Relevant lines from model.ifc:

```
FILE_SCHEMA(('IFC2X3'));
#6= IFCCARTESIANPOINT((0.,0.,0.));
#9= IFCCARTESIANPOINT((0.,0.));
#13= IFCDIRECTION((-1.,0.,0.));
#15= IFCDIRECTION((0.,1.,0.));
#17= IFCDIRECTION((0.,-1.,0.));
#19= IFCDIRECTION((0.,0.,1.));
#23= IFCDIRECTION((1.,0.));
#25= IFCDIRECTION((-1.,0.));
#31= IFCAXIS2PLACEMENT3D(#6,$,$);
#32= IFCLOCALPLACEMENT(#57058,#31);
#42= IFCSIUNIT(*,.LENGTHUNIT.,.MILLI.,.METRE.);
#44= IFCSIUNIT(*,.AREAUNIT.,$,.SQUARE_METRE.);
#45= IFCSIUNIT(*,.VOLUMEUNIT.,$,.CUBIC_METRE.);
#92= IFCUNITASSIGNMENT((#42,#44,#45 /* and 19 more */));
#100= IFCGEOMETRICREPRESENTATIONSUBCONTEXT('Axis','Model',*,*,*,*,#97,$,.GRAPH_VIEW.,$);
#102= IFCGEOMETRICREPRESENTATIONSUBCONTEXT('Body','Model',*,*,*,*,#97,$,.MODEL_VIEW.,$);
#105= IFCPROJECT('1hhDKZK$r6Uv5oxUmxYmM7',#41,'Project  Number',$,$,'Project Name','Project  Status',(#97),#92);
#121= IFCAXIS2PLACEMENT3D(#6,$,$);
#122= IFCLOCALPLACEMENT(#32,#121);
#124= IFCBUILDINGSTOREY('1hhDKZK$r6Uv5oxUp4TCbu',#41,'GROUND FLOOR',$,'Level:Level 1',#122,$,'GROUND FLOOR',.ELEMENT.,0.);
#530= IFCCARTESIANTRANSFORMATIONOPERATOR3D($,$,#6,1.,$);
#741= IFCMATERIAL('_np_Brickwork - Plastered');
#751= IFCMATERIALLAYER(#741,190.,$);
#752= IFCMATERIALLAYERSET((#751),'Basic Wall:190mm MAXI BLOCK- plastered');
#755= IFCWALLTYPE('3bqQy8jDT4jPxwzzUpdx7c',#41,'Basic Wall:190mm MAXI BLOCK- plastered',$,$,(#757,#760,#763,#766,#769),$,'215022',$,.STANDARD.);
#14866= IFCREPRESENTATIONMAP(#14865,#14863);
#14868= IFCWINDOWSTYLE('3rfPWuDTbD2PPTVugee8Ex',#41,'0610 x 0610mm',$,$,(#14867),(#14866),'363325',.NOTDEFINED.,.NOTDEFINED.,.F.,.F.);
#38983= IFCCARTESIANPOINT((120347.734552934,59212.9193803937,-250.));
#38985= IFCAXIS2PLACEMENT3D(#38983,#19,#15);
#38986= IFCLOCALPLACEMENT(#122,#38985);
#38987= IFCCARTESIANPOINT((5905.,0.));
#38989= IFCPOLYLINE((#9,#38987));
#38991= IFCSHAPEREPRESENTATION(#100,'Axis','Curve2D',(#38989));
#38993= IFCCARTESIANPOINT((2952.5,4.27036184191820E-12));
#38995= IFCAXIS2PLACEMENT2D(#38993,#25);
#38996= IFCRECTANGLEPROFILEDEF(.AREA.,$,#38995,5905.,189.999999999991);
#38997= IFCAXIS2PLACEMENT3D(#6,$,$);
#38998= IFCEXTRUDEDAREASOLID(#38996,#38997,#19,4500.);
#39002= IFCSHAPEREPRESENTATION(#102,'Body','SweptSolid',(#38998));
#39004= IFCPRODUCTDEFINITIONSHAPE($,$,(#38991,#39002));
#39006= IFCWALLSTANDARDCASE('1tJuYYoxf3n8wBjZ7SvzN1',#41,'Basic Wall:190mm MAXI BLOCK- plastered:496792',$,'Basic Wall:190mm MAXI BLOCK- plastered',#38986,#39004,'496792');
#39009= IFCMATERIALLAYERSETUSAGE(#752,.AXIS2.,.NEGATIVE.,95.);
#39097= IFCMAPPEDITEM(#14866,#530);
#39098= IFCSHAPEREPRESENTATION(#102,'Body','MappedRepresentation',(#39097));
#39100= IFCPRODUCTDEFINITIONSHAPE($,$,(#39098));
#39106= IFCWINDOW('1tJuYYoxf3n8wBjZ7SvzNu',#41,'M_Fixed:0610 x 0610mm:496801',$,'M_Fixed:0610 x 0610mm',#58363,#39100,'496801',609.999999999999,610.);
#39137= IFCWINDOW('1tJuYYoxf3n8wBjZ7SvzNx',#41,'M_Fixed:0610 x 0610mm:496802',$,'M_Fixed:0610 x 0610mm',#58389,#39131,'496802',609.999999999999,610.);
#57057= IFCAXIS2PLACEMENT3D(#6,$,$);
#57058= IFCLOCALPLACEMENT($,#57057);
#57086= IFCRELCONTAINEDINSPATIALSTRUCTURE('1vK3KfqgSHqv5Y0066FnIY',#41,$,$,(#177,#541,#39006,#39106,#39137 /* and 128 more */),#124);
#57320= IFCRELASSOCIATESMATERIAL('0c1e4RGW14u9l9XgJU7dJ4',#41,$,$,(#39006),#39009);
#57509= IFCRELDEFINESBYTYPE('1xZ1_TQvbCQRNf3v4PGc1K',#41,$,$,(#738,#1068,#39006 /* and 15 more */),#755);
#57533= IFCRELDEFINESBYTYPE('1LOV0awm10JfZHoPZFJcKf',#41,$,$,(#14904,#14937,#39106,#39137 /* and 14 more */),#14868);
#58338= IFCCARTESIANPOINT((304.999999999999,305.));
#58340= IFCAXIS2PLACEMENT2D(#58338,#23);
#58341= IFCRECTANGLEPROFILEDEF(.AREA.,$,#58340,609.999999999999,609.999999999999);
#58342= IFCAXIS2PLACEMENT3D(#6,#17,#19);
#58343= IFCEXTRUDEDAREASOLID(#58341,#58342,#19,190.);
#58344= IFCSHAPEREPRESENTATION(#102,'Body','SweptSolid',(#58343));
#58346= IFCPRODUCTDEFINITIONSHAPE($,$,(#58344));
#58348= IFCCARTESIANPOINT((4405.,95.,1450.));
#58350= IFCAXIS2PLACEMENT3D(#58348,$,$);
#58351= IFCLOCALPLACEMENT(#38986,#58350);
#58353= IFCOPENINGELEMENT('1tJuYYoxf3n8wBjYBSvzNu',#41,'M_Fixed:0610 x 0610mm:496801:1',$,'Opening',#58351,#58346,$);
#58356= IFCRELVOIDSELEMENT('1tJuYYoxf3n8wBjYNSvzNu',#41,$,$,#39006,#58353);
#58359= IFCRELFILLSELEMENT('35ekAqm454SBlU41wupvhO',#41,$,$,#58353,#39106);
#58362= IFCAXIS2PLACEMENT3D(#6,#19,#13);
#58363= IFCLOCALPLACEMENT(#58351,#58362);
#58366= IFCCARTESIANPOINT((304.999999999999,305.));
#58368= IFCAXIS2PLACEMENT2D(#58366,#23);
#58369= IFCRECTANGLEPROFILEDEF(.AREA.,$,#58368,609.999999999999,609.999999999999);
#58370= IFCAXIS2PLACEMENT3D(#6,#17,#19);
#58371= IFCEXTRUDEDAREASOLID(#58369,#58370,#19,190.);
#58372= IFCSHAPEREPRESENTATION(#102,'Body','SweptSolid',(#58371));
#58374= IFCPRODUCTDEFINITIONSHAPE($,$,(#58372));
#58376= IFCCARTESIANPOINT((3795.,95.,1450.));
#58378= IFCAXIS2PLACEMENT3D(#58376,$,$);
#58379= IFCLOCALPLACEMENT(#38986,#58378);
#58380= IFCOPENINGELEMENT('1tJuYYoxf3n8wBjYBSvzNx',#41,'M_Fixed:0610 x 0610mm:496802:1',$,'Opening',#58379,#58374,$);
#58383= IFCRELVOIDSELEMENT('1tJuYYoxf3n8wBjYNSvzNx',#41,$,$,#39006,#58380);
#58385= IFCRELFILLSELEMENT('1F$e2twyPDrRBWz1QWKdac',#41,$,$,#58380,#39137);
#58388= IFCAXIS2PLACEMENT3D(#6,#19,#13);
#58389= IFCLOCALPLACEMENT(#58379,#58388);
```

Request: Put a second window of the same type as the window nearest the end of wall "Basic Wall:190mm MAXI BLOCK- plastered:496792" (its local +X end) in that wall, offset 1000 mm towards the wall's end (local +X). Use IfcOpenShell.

```python
import ifcopenshell
import ifcopenshell.api.feature
import ifcopenshell.api.geometry
import ifcopenshell.api.root
import ifcopenshell.geom
import ifcopenshell.util.element
import ifcopenshell.util.placement
import ifcopenshell.util.shape

model = ifcopenshell.open("model.ifc")
settings = ifcopenshell.geom.settings()


def volume(element):
    """Net volume in cubic metres, openings subtracted."""
    shape = ifcopenshell.geom.create_shape(settings, element)
    return ifcopenshell.util.shape.get_volume(shape.geometry)


def reuse_history(source, copy):
    """copy_class also copies each property set's owner history, people and application; keep the originals."""
    for rel in copy.IsDefinedBy:
        if rel.is_a("IfcRelDefinesByProperties") and (history := rel.RelatingPropertyDefinition.OwnerHistory):
            rel.RelatingPropertyDefinition.OwnerHistory = source.OwnerHistory
            ifcopenshell.util.element.remove_deep2(model, history)


window = model.by_guid("1tJuYYoxf3n8wBjZ7SvzNu")
opening = window.FillsVoids[0].RelatingOpeningElement
wall = opening.VoidsElements[0].RelatingBuildingElement
before = volume(wall)
shift = ifcopenshell.util.placement.get_local_placement(wall.ObjectPlacement)[:3, 0] * 1000.0

# copy_class copies the void relationship, type, container and properties, but no geometry.
new_opening = ifcopenshell.api.root.copy_class(model, product=opening)
new_opening.Representation = ifcopenshell.util.element.copy_deep(
    model, opening.Representation, exclude=["IfcGeometricRepresentationContext", "IfcRepresentationMap"]
)
new_opening.Name = "M_Fixed:0610 x 0610mm"
new_window = ifcopenshell.api.root.copy_class(model, product=window)
new_window.Representation = ifcopenshell.util.element.copy_deep(
    model, window.Representation, exclude=["IfcGeometricRepresentationContext", "IfcRepresentationMap"]
)
new_window.Name = "M_Fixed:0610 x 0610mm"
new_window.Tag = None
reuse_history(window, new_window)
fills = ifcopenshell.api.feature.add_filling(model, opening=new_opening, element=new_window)
fills.OwnerHistory = new_window.OwnerHistory  # required in IFC2X3

for old, new in ((opening, new_opening), (window, new_window)):
    matrix = ifcopenshell.util.placement.get_local_placement(old.ObjectPlacement)
    matrix[:3, 3] += shift
    ifcopenshell.api.geometry.edit_object_placement(model, product=new, matrix=matrix, is_si=False)

after = volume(wall)

print(f"wall volume {before:.3f} -> {after:.3f} m3")

model.write("model_rev.ifc")
```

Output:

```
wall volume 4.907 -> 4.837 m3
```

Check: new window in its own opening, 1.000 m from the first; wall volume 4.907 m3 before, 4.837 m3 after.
